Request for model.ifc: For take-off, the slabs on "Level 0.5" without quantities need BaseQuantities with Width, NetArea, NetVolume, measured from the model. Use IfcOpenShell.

First a look at what the model holds.

```python
import ifcopenshell
import ifcopenshell.util.element
import ifcopenshell.util.unit

model = ifcopenshell.open("model.ifc")
print(model.schema)
for unit_type in ("LENGTHUNIT", "AREAUNIT", "VOLUMEUNIT"):
    print(unit_type, ifcopenshell.util.unit.calculate_unit_scale(model, unit_type))
storey = next(s for s in model.by_type("IfcBuildingStorey") if s.Name == "Level 0.5")
slabs = [e for e in ifcopenshell.util.element.get_decomposition(storey) if e.is_a("IfcSlab")]
for e in sorted(slabs, key=lambda e: e.id()):
    print(e.id(), e.is_a(), e.Name, list(ifcopenshell.util.element.get_psets(e, qtos_only=True)), sep=" | ")
```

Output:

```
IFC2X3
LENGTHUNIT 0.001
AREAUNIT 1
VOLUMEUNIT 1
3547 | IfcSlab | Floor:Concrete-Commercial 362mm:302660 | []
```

```python
import ifcopenshell
import ifcopenshell.api.pset
import ifcopenshell.geom
import ifcopenshell.util.element
import ifcopenshell.util.shape
import ifcopenshell.util.unit

model = ifcopenshell.open("model.ifc")
unit_scale = ifcopenshell.util.unit.calculate_unit_scale(model)
area_scale = ifcopenshell.util.unit.calculate_unit_scale(model, "AREAUNIT")
volume_scale = ifcopenshell.util.unit.calculate_unit_scale(model, "VOLUMEUNIT")
settings = ifcopenshell.geom.settings()

storey = next(s for s in model.by_type("IfcBuildingStorey") if s.Name == "Level 0.5")
slabs = [e for e in ifcopenshell.util.element.get_decomposition(storey) if e.is_a("IfcSlab")]

for e in sorted(slabs, key=lambda e: e.id()):
    if ifcopenshell.util.element.get_psets(e, qtos_only=True, should_inherit=False):
        continue
    # Geometry comes back in metres, in the element's own axes.
    shape = ifcopenshell.geom.create_shape(settings, e)
    values = {
        "Width": ifcopenshell.util.shape.get_z(shape.geometry) / unit_scale,
        "NetArea": ifcopenshell.util.shape.get_footprint_area(shape.geometry) / area_scale,
        "NetVolume": ifcopenshell.util.shape.get_volume(shape.geometry) / volume_scale,
    }
    qto = ifcopenshell.api.pset.add_qto(model, product=e, name="BaseQuantities")
    ifcopenshell.api.pset.edit_qto(model, qto=qto, properties=values)
    print(e.id(), {k: round(v, 3) for k, v in values.items()})

model.write("model_updated.ifc")
```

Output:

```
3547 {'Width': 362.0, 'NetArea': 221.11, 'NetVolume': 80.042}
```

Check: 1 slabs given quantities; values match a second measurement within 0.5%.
